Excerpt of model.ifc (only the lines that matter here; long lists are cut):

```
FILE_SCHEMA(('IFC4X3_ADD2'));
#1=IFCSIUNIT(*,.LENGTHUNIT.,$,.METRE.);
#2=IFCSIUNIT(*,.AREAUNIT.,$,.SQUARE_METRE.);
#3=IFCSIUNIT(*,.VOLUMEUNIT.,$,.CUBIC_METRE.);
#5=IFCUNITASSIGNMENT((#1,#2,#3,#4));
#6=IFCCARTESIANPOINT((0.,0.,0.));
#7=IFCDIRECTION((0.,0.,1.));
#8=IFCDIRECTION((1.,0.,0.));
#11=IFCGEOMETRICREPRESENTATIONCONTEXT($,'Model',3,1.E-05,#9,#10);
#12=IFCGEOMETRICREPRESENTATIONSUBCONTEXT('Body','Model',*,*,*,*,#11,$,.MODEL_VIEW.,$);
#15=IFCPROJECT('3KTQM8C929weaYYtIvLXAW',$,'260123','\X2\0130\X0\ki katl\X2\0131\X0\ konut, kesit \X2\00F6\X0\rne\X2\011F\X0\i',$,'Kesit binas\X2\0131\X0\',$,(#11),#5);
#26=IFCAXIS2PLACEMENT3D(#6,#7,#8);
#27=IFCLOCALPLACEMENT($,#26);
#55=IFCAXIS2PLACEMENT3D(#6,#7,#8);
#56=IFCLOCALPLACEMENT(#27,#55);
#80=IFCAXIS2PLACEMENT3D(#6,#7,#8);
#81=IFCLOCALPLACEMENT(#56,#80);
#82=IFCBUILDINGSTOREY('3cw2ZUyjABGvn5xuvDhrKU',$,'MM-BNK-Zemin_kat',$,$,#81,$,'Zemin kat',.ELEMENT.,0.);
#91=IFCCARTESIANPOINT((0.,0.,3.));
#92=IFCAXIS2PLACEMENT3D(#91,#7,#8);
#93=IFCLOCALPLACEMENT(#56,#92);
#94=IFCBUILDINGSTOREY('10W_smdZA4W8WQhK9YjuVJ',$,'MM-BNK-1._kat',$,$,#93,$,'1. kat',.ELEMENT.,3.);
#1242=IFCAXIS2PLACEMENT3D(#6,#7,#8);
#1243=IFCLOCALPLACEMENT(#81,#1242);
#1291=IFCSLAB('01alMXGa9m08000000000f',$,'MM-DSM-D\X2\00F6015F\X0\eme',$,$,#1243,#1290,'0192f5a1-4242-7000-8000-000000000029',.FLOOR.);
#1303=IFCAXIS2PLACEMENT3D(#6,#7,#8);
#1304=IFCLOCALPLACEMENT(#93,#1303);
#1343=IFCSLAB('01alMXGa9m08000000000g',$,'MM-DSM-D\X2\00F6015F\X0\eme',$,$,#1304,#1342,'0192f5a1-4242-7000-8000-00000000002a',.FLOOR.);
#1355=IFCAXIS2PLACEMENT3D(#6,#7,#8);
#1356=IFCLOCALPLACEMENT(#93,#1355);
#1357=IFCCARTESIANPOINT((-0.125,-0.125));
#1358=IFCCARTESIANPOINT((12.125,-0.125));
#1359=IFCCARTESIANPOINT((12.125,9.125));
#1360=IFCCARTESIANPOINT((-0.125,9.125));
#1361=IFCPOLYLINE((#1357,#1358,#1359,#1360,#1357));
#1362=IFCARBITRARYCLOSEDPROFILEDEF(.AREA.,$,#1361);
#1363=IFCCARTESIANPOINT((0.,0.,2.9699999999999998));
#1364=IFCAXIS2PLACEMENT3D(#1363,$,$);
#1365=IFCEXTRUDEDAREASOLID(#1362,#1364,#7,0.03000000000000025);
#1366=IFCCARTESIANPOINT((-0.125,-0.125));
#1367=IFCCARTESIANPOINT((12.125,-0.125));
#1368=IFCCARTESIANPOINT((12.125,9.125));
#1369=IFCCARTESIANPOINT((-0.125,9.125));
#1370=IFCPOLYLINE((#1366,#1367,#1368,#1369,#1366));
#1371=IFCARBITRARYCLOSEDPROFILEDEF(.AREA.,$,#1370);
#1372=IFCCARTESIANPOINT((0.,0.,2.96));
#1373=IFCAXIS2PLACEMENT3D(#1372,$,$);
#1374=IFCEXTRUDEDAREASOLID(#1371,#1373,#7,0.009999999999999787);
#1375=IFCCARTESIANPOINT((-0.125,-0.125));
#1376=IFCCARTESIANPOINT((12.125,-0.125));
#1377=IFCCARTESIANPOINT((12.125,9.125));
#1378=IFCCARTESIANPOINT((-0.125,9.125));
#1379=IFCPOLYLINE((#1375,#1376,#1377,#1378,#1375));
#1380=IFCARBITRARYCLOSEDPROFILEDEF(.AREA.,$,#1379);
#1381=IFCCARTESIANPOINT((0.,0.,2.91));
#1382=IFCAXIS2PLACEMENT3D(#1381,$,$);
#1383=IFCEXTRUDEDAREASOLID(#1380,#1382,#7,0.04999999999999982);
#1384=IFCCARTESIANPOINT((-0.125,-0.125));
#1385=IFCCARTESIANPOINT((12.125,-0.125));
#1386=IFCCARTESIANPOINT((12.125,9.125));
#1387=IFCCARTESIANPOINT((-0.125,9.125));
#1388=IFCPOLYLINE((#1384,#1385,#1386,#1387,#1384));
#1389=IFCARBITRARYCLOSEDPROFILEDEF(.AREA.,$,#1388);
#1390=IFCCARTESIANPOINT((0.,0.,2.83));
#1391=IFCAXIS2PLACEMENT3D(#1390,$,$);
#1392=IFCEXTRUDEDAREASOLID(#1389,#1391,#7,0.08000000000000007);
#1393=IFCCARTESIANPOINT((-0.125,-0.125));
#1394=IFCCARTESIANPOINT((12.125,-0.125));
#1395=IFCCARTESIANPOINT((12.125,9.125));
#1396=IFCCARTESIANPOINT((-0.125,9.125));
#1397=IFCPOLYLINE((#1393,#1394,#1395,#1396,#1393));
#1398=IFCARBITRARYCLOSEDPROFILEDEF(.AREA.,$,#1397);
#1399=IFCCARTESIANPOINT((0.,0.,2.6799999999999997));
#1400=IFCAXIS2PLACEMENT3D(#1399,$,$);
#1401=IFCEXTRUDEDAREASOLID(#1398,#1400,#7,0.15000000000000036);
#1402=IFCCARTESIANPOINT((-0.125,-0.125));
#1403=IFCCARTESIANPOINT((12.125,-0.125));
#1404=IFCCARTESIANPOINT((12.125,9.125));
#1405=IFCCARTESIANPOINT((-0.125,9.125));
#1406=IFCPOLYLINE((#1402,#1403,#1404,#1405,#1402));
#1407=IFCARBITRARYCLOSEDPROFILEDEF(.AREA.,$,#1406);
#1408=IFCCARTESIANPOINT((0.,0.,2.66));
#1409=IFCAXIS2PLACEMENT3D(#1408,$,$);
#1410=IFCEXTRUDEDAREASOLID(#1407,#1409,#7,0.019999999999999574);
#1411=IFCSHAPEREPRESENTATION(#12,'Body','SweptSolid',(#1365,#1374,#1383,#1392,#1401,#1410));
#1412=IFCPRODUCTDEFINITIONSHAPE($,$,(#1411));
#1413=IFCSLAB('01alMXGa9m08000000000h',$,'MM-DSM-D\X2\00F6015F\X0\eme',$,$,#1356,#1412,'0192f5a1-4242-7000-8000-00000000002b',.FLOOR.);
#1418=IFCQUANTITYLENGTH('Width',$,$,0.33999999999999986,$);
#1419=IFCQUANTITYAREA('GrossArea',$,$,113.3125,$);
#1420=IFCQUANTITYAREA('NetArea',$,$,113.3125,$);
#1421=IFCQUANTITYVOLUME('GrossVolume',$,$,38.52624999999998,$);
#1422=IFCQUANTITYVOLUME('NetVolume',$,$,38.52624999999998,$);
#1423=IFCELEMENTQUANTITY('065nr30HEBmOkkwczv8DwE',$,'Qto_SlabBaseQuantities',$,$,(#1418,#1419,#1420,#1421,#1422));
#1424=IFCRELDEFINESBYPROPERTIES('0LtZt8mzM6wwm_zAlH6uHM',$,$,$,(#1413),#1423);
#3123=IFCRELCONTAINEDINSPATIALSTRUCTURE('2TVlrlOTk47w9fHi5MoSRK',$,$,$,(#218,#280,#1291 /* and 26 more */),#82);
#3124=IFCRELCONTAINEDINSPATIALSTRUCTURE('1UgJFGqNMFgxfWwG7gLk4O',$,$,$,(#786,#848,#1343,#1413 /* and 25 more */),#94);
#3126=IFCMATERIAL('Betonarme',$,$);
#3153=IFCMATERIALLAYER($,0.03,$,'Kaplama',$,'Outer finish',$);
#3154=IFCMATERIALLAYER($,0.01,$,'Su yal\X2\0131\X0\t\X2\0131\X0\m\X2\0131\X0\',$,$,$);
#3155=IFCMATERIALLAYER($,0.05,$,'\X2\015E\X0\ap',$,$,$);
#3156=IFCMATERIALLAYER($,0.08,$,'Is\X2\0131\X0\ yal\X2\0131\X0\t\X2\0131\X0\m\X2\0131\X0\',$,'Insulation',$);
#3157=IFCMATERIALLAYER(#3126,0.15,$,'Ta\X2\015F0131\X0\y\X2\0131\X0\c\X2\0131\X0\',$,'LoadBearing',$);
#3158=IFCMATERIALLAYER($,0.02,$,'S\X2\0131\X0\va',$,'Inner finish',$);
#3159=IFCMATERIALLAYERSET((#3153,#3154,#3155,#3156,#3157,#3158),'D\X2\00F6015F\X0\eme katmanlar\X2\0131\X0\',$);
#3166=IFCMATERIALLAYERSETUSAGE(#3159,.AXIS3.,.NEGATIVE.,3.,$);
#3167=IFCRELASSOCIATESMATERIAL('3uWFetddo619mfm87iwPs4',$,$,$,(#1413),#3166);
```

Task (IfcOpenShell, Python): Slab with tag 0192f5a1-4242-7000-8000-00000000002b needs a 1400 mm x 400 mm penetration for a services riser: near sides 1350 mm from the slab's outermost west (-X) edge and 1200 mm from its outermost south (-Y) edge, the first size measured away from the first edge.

```python
import numpy as np
import ifcopenshell
import ifcopenshell.api.feature
import ifcopenshell.api.geometry
import ifcopenshell.api.pset
import ifcopenshell.api.root
import ifcopenshell.geom
import ifcopenshell.util.element
import ifcopenshell.util.placement
import ifcopenshell.util.representation
import ifcopenshell.util.shape
import ifcopenshell.util.unit

model = ifcopenshell.open("model.ifc")
unit_scale = ifcopenshell.util.unit.calculate_unit_scale(model)
area_scale = ifcopenshell.util.unit.calculate_unit_scale(model, "AREAUNIT")
volume_scale = ifcopenshell.util.unit.calculate_unit_scale(model, "VOLUMEUNIT")
settings = ifcopenshell.geom.settings()


def volume(element):
    """Net volume in cubic metres, openings subtracted."""
    shape = ifcopenshell.geom.create_shape(settings, element)
    return ifcopenshell.util.shape.get_volume(shape.geometry)


slab = model.by_guid("01alMXGa9m08000000000h")
before = volume(slab)

# Extent in the slab's own axes, in metres. The edges named are its -X and -Y sides.
slab_shape = ifcopenshell.geom.create_shape(settings, slab)
vertices = ifcopenshell.util.shape.get_vertices(slab_shape.geometry)
x_min, y_min, bottom = vertices.min(axis=0)
top = vertices[:, 2].max()

opening = ifcopenshell.api.root.create_entity(model, ifc_class="IfcOpeningElement", name="Services riser opening", predefined_type="OPENING")
context = ifcopenshell.util.representation.get_context(model, "Model", "Body", "MODEL_VIEW")
width, depth = 1.4, 0.4
outline = [(0.0, 0.0), (width, 0.0), (width, depth), (0.0, depth), (0.0, 0.0)]
# Overshoot both faces by 50 mm so the cut is clean.
shape = ifcopenshell.api.geometry.add_slab_representation(
    model, context=context, depth=top - bottom + 0.1, polyline=outline
)
ifcopenshell.api.geometry.assign_representation(model, product=opening, representation=shape)

matrix = ifcopenshell.util.placement.get_local_placement(slab.ObjectPlacement)
matrix[:, 3] = matrix @ np.append(np.array([x_min + 1.35, y_min + 1.2, bottom - 0.05]) / unit_scale, 1.0)
ifcopenshell.api.geometry.edit_object_placement(model, product=opening, matrix=matrix, is_si=False)
ifcopenshell.api.feature.add_feature(model, feature=opening, element=slab)

after = volume(slab)

# Update the slab's stored quantities.
qto = model.by_id(ifcopenshell.util.element.get_pset(slab, "Qto_SlabBaseQuantities", should_inherit=False)["id"])
ifcopenshell.api.pset.edit_qto(model, qto=qto, properties={
    "NetArea": after / (top - bottom) / area_scale,
    "NetVolume": after / volume_scale,
})

print(f"slab volume {before:.3f} -> {after:.3f} m3")

model.write("model_updated.ifc")
```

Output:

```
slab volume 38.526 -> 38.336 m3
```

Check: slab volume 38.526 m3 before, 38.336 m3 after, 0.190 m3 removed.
